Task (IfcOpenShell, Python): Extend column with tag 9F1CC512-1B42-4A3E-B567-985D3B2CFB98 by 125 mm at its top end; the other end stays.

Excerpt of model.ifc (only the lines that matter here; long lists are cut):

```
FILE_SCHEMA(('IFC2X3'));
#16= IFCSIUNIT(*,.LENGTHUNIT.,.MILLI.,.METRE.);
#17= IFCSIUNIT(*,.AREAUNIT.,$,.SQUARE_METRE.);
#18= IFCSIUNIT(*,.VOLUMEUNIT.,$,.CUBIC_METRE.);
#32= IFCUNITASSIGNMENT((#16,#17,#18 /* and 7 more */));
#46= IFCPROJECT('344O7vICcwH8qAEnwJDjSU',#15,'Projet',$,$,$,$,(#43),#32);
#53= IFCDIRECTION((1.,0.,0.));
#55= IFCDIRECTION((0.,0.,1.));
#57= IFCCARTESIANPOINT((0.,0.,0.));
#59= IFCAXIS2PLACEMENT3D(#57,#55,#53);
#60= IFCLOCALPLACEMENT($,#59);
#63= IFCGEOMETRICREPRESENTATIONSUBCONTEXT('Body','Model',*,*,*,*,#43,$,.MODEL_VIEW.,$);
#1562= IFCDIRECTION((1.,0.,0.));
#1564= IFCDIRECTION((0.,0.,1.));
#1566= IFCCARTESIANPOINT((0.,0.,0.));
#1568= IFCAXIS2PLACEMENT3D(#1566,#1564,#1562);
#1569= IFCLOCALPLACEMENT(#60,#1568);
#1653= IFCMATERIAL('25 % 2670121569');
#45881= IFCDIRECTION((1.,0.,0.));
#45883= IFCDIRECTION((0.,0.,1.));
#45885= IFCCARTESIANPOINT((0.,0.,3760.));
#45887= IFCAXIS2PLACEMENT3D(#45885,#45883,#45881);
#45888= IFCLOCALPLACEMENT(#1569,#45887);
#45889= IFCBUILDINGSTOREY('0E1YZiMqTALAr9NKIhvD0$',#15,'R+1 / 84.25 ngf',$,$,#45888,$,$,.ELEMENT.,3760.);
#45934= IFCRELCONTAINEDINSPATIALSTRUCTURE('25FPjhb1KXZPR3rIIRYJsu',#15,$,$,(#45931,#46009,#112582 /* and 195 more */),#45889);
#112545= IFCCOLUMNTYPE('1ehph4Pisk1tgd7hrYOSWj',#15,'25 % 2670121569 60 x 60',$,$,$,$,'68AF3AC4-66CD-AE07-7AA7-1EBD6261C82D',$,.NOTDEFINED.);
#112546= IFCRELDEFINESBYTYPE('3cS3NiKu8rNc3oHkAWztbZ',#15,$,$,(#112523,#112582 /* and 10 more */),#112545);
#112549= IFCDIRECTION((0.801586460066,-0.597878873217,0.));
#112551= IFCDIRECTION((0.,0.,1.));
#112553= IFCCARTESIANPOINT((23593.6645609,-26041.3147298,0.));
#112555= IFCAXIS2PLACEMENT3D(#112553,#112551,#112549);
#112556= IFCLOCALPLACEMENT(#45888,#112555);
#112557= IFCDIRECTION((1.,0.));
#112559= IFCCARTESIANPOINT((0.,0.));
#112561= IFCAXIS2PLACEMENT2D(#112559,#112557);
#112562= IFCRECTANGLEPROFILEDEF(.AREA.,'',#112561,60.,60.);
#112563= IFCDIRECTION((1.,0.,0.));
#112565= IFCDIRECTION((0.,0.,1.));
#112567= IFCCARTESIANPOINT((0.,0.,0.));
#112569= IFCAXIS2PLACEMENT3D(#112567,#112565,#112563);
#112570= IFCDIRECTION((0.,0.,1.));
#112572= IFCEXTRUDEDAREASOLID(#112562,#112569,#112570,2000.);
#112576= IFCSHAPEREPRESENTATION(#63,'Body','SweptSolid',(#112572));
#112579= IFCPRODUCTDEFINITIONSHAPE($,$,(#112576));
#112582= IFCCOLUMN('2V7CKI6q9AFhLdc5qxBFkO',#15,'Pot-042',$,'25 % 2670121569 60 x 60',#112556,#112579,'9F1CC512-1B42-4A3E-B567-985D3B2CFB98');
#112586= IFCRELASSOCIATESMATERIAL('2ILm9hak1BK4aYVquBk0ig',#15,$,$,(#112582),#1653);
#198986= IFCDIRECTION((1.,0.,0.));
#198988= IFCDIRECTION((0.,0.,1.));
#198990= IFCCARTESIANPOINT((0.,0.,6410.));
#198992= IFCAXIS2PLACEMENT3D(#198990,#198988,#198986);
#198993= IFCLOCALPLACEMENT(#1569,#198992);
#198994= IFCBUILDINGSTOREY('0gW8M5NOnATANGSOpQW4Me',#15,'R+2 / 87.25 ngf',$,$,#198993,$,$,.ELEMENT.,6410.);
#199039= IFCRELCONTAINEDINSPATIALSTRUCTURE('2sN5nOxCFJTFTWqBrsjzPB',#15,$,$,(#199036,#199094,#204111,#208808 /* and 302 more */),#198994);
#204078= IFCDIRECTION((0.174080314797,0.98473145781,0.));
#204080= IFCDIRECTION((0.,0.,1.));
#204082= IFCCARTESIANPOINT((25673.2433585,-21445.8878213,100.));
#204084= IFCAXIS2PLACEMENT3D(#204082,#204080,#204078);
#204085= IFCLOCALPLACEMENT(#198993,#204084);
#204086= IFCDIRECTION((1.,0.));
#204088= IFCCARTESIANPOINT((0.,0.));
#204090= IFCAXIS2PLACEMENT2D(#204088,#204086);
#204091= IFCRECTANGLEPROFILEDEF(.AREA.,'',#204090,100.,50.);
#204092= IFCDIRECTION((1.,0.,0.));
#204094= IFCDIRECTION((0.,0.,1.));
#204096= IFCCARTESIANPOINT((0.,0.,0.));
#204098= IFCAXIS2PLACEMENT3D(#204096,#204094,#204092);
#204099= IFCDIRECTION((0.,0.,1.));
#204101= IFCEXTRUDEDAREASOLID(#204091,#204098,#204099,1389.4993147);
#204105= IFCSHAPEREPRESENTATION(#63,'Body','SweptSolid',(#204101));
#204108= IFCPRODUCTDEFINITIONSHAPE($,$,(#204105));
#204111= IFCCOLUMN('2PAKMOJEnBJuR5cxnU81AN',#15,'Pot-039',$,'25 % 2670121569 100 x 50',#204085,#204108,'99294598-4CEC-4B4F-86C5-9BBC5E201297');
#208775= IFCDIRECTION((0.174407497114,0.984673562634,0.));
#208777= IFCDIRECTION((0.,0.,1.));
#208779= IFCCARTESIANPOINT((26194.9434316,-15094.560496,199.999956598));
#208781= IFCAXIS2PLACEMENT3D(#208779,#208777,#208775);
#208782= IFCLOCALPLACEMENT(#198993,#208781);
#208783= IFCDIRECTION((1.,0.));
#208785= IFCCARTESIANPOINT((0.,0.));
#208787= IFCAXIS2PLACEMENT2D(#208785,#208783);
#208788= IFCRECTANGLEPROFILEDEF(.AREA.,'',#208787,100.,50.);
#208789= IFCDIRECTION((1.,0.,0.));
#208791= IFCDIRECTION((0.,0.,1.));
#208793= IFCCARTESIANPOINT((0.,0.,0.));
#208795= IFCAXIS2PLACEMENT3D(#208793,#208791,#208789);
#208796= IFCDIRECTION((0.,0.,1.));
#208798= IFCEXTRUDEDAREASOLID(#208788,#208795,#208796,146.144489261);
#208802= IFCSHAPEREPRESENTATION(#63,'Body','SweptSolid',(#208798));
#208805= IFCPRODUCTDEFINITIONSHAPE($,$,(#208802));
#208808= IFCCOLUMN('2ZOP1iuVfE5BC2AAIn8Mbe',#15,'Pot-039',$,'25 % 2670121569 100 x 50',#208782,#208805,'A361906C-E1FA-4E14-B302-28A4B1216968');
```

```python
import ifcopenshell
import ifcopenshell.util.representation

model = ifcopenshell.open("model.ifc")

member = model.by_id(112582)
change = 125.0

# The extrusion runs towards the end named, so only its depth changes.
body = ifcopenshell.util.representation.get_representation(member, "Model", "Body")
solid = body.Items[0]
old_length = solid.Depth
solid.Depth += change

print(f"length {old_length:g} -> {solid.Depth:g}")

model.write("model_v2.ifc")
```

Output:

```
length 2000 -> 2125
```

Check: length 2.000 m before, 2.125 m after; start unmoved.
